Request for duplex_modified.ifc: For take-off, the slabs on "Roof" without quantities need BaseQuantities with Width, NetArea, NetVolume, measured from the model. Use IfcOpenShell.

First a look at what the model holds.

```python
import ifcopenshell
import ifcopenshell.util.element
import ifcopenshell.util.unit

model = ifcopenshell.open("duplex_modified.ifc")
print(model.schema)
for unit_type in ("LENGTHUNIT", "AREAUNIT", "VOLUMEUNIT"):
    print(unit_type, ifcopenshell.util.unit.calculate_unit_scale(model, unit_type))
storey = next(s for s in model.by_type("IfcBuildingStorey") if s.Name == "Roof")
slabs = [e for e in ifcopenshell.util.element.get_decomposition(storey) if e.is_a("IfcSlab")]
for e in sorted(slabs, key=lambda e: e.id()):
    print(e.id(), e.is_a(), e.Name, list(ifcopenshell.util.element.get_psets(e, qtos_only=True)), sep=" | ")
```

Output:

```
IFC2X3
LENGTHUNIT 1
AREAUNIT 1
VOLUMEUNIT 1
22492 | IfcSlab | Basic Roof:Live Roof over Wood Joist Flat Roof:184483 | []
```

```python
import ifcopenshell
import ifcopenshell.api.pset
import ifcopenshell.geom
import ifcopenshell.util.element
import ifcopenshell.util.shape
import ifcopenshell.util.unit

model = ifcopenshell.open("duplex_modified.ifc")
unit_scale = ifcopenshell.util.unit.calculate_unit_scale(model)
area_scale = ifcopenshell.util.unit.calculate_unit_scale(model, "AREAUNIT")
volume_scale = ifcopenshell.util.unit.calculate_unit_scale(model, "VOLUMEUNIT")
settings = ifcopenshell.geom.settings()

storey = next(s for s in model.by_type("IfcBuildingStorey") if s.Name == "Roof")
slabs = [e for e in ifcopenshell.util.element.get_decomposition(storey) if e.is_a("IfcSlab")]

for e in sorted(slabs, key=lambda e: e.id()):
    if ifcopenshell.util.element.get_psets(e, qtos_only=True, should_inherit=False):
        continue
    # Geometry comes back in metres, in the element's own axes.
    shape = ifcopenshell.geom.create_shape(settings, e)
    values = {
        "Width": ifcopenshell.util.shape.get_z(shape.geometry) / unit_scale,
        "NetArea": ifcopenshell.util.shape.get_footprint_area(shape.geometry) / area_scale,
        "NetVolume": ifcopenshell.util.shape.get_volume(shape.geometry) / volume_scale,
    }
    qto = ifcopenshell.api.pset.add_qto(model, product=e, name="BaseQuantities")
    ifcopenshell.api.pset.edit_qto(model, qto=qto, properties=values)
    print(e.id(), {k: round(v, 3) for k, v in values.items()})

model.write("duplex_modified_edited.ifc")
```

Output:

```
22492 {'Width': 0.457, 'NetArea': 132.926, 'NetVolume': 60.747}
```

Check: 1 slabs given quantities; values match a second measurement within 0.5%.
